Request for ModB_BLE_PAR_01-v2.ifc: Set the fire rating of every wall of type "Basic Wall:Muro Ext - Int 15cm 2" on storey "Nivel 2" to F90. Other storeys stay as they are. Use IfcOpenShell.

First a look at what the model holds.

```python
import ifcopenshell
import ifcopenshell.util.element

model = ifcopenshell.open("ModB_BLE_PAR_01-v2.ifc")
print(model.schema)
storey = next(s for s in model.by_type("IfcBuildingStorey") if s.Name == "Nivel 2")
walls = [e for e in ifcopenshell.util.element.get_decomposition(storey) if e.is_a("IfcWall")]
seen = {}
for e in walls:
    element_type = ifcopenshell.util.element.get_type(e)
    key = (element_type.Name if element_type != e and element_type else None, ifcopenshell.util.element.get_pset(e, "Pset_WallCommon", "FireRating"))
    seen[key] = seen.get(key, 0) + 1
for (name, value), count in sorted(seen.items(), key=str):
    print(count, "x", name, "|", value)
```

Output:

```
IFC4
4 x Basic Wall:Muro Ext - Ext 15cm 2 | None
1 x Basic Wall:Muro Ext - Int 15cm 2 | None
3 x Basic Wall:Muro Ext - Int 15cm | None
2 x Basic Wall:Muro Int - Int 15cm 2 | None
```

```python
import ifcopenshell
import ifcopenshell.api.pset
import ifcopenshell.util.element

model = ifcopenshell.open("ModB_BLE_PAR_01-v2.ifc")

storey = next(s for s in model.by_type("IfcBuildingStorey") if s.Name == "Nivel 2")
walls = [e for e in ifcopenshell.util.element.get_decomposition(storey) if e.is_a("IfcWall")]

count = 0
for e in walls:
    element_type = ifcopenshell.util.element.get_type(e)
    if element_type in (None, e) or element_type.Name != "Basic Wall:Muro Ext - Int 15cm 2":
        continue
    # add_pset returns the element's existing set when there is one.
    pset = ifcopenshell.api.pset.add_pset(model, product=e, name="Pset_WallCommon")
    ifcopenshell.api.pset.edit_pset(model, pset=pset, properties={"FireRating": "F90"})
    count += 1

print(count, "walls updated")

model.write("ModB_BLE_PAR_01-v2_v2.ifc")
```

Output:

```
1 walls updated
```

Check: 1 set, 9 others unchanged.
